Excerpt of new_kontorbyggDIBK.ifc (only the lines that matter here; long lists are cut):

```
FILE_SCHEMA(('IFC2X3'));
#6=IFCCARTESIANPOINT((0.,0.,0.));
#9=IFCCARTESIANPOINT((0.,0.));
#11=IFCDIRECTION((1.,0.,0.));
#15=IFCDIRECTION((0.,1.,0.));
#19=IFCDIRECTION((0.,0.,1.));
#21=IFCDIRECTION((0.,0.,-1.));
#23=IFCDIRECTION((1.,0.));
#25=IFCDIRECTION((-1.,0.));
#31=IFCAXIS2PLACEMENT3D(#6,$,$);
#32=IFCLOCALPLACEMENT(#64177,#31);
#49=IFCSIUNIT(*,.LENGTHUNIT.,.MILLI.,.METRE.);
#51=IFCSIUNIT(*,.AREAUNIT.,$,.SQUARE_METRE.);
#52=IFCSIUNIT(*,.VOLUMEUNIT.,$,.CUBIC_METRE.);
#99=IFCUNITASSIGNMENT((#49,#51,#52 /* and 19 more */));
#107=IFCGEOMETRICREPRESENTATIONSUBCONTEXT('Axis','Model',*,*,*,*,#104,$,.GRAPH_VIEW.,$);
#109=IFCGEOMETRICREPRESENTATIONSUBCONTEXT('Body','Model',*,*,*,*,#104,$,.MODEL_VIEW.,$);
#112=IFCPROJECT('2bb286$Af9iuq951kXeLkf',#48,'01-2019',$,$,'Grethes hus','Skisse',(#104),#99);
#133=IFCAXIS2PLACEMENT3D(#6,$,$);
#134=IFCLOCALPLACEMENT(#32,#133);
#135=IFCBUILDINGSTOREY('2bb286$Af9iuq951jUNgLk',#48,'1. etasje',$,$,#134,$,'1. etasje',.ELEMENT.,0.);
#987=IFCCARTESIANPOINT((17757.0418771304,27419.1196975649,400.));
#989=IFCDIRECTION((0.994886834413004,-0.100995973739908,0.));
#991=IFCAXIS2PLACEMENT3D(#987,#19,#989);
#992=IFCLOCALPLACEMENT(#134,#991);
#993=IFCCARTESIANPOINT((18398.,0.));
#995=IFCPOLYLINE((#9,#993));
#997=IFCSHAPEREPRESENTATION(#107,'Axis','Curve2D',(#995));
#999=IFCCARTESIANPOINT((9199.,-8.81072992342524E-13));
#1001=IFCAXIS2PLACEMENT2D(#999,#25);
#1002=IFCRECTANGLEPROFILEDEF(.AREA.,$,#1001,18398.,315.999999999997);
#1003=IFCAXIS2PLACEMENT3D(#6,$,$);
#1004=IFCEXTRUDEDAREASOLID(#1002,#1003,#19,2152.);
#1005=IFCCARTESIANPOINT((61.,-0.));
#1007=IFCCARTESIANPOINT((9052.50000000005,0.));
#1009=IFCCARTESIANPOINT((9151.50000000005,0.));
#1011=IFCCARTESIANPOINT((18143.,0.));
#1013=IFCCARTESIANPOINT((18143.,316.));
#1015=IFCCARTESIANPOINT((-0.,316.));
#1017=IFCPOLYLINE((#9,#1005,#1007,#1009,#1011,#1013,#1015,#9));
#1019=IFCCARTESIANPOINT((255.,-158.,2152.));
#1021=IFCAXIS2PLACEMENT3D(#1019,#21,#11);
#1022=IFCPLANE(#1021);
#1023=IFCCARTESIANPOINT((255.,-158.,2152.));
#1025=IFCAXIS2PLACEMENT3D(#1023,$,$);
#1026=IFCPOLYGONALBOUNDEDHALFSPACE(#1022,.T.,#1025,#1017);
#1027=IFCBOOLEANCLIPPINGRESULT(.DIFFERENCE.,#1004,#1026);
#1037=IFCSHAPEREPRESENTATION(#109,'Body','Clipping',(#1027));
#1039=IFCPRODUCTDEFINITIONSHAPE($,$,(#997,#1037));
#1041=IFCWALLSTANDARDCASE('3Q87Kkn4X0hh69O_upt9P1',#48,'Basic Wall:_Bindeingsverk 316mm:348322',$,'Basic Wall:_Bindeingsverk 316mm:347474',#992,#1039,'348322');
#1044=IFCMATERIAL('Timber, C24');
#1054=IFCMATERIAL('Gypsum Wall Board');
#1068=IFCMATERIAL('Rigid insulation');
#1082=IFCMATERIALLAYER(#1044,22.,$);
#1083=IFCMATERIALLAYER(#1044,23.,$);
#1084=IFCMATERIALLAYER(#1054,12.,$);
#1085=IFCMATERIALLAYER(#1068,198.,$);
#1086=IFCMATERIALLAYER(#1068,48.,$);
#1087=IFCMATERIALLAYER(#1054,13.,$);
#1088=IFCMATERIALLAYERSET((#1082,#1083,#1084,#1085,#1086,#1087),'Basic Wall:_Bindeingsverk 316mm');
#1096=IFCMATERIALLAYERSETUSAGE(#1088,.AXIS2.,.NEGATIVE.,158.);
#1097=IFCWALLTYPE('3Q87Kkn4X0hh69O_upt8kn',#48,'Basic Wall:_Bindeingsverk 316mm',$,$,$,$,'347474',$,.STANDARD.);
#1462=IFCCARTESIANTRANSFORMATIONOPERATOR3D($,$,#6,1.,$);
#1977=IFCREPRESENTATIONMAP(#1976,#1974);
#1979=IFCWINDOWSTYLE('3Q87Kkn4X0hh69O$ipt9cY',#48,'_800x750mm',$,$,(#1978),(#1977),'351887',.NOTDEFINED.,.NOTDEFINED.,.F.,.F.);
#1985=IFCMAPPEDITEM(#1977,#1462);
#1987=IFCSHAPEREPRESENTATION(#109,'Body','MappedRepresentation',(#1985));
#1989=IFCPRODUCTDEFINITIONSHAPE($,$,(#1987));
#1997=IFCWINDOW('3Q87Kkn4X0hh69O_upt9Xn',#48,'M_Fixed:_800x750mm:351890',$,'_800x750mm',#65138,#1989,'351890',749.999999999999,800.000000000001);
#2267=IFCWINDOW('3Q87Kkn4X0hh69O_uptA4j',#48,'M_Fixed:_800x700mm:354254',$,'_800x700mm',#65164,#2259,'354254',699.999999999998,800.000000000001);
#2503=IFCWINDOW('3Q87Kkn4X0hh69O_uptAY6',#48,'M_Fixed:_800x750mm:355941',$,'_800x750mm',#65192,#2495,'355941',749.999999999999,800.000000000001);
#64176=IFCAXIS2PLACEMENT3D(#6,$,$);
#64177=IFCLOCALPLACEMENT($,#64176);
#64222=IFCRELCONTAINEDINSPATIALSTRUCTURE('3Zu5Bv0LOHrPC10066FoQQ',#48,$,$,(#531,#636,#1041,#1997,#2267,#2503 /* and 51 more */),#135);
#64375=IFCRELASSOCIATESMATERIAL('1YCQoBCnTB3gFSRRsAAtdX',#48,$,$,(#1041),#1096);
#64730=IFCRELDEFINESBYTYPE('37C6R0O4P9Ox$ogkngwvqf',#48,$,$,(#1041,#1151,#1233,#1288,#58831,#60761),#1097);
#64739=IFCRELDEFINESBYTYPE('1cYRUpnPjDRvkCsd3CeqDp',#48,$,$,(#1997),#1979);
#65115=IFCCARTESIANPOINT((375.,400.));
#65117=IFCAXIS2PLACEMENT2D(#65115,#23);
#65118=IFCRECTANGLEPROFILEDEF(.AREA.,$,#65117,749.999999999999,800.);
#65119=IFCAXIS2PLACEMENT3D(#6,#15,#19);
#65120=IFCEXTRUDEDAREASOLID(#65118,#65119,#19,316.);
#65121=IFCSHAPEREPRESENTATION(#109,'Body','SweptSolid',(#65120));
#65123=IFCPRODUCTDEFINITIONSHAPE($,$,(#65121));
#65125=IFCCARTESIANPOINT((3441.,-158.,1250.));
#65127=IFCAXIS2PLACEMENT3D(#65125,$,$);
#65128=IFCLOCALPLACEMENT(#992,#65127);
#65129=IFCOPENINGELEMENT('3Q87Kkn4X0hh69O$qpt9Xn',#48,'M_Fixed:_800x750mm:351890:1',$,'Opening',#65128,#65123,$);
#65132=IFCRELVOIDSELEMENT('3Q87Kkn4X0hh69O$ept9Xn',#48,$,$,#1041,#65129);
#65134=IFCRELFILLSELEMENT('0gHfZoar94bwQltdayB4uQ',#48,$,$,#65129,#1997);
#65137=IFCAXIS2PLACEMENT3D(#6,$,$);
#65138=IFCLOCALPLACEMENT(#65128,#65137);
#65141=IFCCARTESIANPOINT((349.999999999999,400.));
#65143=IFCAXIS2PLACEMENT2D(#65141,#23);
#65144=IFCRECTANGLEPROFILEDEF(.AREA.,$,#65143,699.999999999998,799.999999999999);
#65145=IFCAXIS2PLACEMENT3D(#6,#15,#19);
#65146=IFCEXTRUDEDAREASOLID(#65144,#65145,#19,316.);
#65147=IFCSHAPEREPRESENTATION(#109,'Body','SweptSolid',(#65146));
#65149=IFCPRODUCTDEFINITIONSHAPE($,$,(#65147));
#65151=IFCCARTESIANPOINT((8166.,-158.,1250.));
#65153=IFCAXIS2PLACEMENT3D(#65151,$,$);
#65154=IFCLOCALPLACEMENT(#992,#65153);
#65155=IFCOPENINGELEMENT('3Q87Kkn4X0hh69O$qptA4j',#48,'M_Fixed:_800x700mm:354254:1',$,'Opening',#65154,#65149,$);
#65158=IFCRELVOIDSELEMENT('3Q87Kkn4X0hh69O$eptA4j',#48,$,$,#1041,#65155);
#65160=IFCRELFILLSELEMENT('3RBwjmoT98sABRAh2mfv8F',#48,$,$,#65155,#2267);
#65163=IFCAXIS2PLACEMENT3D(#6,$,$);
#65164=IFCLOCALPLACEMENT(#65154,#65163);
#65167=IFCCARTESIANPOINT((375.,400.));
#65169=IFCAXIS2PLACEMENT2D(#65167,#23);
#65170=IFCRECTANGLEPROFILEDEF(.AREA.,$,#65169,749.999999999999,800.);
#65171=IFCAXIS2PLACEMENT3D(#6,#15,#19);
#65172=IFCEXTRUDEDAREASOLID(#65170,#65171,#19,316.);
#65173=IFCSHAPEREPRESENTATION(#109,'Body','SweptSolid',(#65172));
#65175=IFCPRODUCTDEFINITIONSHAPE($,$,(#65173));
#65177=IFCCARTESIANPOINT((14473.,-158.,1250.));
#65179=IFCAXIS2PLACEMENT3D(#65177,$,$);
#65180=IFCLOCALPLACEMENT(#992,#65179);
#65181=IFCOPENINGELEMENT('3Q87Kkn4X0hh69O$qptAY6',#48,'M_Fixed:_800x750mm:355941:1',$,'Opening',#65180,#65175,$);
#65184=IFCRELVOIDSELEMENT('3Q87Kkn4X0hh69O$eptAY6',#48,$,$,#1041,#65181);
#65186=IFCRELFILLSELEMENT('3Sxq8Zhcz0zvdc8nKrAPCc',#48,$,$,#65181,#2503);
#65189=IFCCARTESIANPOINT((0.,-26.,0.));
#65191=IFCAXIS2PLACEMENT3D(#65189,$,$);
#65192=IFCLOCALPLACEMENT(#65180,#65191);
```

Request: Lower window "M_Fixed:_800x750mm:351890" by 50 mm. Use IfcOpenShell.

```python
import numpy as np
import ifcopenshell
import ifcopenshell.api.geometry
import ifcopenshell.util.placement
import ifcopenshell.util.unit

model = ifcopenshell.open("new_kontorbyggDIBK.ifc")
unit_scale = ifcopenshell.util.unit.calculate_unit_scale(model)

window = model.by_guid("3Q87Kkn4X0hh69O_upt9Xn")
opening = window.FillsVoids[0].RelatingOpeningElement
dz = -0.05 / unit_scale

shift = np.array([0.0, 0.0, dz])
# The window is placed relative to its opening, so it follows when the opening moves.
matrix = ifcopenshell.util.placement.get_local_placement(opening.ObjectPlacement)
matrix[:3, 3] += shift
ifcopenshell.api.geometry.edit_object_placement(
    model, product=opening, matrix=matrix, is_si=False, should_transform_children=True
)

print(f"moved by {dz * unit_scale:+.3f} m")

model.write("new_kontorbyggDIBK_updated.ifc")
```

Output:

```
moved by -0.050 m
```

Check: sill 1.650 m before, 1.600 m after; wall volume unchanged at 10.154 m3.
